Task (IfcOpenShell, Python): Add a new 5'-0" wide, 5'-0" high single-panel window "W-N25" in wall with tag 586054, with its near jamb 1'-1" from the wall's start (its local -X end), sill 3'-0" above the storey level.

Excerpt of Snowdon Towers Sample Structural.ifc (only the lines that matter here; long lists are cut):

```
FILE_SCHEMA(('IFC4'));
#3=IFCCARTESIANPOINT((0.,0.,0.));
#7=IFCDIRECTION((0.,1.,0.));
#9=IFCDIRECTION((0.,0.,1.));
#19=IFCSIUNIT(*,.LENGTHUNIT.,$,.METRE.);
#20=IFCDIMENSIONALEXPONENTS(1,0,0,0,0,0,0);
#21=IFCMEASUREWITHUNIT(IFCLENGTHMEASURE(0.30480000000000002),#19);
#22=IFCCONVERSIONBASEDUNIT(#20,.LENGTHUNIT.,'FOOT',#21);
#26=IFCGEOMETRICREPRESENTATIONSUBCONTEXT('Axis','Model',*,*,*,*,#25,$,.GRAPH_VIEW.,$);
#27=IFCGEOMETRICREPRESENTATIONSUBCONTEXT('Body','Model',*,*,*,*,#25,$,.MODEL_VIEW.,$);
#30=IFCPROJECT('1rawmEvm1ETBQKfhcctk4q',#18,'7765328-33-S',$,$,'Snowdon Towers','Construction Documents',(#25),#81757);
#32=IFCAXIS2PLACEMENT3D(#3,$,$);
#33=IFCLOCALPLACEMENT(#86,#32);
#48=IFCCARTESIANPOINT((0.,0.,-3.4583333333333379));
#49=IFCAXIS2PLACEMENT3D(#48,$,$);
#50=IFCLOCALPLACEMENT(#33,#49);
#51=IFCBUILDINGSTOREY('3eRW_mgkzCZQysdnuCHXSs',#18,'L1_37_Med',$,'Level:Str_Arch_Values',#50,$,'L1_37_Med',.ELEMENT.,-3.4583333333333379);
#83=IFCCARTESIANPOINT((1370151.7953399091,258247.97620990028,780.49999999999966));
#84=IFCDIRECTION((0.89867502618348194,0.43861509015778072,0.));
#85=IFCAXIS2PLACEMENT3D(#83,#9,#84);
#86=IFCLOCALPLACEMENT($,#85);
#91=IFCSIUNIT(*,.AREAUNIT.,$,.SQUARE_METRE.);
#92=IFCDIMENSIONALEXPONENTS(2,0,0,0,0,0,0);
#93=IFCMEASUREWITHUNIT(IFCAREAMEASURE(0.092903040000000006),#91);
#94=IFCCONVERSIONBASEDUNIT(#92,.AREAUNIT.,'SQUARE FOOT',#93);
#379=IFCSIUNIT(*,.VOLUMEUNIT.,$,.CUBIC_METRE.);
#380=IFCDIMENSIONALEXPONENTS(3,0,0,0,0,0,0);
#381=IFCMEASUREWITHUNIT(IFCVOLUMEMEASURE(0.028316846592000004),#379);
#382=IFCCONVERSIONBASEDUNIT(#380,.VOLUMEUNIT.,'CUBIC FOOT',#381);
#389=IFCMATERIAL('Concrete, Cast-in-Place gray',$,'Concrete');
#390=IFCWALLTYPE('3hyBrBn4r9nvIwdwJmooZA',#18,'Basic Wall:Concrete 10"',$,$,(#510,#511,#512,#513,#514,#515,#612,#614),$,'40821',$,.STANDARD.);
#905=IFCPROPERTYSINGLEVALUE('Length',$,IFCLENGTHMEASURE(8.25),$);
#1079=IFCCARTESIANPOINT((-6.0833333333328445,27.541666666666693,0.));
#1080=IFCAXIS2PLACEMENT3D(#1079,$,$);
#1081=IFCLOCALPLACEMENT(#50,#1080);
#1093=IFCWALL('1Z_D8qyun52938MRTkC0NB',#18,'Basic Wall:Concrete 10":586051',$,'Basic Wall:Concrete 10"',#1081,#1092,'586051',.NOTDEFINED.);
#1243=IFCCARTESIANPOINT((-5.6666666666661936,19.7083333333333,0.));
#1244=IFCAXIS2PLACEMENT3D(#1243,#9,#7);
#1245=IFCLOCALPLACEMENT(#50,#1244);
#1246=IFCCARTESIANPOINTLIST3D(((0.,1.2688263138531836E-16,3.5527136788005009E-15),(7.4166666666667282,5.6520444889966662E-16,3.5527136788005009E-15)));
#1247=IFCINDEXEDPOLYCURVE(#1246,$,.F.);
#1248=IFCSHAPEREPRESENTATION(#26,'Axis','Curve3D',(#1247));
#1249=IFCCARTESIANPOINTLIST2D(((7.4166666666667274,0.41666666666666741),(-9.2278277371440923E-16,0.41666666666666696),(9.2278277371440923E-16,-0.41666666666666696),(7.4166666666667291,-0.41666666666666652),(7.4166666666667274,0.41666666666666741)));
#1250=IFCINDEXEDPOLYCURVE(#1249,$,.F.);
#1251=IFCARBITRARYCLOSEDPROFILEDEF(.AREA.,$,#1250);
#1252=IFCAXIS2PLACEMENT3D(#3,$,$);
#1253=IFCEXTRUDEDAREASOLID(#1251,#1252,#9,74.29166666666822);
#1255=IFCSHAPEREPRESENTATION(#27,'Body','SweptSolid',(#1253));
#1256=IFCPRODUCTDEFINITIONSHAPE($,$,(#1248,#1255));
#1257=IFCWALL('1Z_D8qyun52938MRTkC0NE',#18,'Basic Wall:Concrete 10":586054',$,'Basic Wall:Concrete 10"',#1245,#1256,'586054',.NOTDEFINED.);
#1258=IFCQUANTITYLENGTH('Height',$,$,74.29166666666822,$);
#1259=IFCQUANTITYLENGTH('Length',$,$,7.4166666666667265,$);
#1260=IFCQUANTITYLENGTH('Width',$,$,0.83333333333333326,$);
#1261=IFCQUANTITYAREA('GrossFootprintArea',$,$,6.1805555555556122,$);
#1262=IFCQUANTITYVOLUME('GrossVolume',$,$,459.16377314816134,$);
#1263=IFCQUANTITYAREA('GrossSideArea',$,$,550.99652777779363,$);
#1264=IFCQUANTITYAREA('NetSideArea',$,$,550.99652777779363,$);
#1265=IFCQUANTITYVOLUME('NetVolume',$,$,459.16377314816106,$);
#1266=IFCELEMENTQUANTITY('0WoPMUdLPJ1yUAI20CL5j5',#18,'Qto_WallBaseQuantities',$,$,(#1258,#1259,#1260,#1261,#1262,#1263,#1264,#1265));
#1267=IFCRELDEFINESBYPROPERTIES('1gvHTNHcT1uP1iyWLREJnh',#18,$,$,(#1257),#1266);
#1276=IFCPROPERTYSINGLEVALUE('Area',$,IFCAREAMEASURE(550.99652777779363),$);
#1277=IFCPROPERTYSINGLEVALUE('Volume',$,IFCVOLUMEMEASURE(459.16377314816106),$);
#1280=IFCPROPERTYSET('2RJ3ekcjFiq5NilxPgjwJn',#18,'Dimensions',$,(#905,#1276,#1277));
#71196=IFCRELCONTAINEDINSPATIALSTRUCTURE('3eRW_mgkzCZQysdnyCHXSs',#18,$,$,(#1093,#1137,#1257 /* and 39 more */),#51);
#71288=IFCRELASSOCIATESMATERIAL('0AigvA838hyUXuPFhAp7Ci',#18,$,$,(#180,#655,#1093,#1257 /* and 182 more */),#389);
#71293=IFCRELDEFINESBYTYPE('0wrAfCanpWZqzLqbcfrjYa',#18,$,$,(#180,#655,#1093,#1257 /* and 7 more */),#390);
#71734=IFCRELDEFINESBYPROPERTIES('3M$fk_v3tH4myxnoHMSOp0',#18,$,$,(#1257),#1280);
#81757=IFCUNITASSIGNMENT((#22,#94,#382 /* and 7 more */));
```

```python
import numpy as np
import ifcopenshell
import ifcopenshell.api.feature
import ifcopenshell.api.geometry
import ifcopenshell.api.pset
import ifcopenshell.api.root
import ifcopenshell.api.spatial
import ifcopenshell.geom
import ifcopenshell.util.element
import ifcopenshell.util.placement
import ifcopenshell.util.representation
import ifcopenshell.util.shape
import ifcopenshell.util.unit

model = ifcopenshell.open("Snowdon Towers Sample Structural.ifc")
unit_scale = ifcopenshell.util.unit.calculate_unit_scale(model)
area_scale = ifcopenshell.util.unit.calculate_unit_scale(model, "AREAUNIT")
volume_scale = ifcopenshell.util.unit.calculate_unit_scale(model, "VOLUMEUNIT")
settings = ifcopenshell.geom.settings()


def volume(element):
    """Net volume in cubic metres, openings subtracted."""
    shape = ifcopenshell.geom.create_shape(settings, element)
    return ifcopenshell.util.shape.get_volume(shape.geometry)


wall = model.by_id(1257)
storey = ifcopenshell.util.element.get_container(wall, ifc_class="IfcBuildingStorey")
context = ifcopenshell.util.representation.get_context(model, "Model", "Body", "MODEL_VIEW")
before = volume(wall)

width, height, from_end, sill = 1.524, 1.524, 0.3302, 0.9144  # metres

# The wall runs along its own X axis, and the end named is its -X end.
wall_shape = ifcopenshell.geom.create_shape(settings, wall)
x, y, z = ifcopenshell.util.shape.get_vertices(wall_shape.geometry).T
start = x.min() + from_end
face, thickness = float(y.min()), float(y.max() - y.min())
wall_matrix = ifcopenshell.util.placement.get_local_placement(wall.ObjectPlacement)
level = ifcopenshell.util.placement.get_local_placement(storey.ObjectPlacement)[2, 3]


def in_wall(x, y):
    """Placement at x, y metres in the wall's axes, at sill height."""
    matrix = wall_matrix.copy()
    matrix[:, 3] = wall_matrix @ np.array([x / unit_scale, y / unit_scale, 0.0, 1.0])
    matrix[2, 3] = level + sill / unit_scale
    return matrix


# Opening: a box that overshoots both wall faces by 50 mm.
opening = ifcopenshell.api.root.create_entity(model, ifc_class="IfcOpeningElement", predefined_type="OPENING")
box = ifcopenshell.api.geometry.add_wall_representation(
    model, context=context, length=width, height=height, thickness=thickness + 0.1
)
ifcopenshell.api.geometry.assign_representation(model, product=opening, representation=box)
ifcopenshell.api.geometry.edit_object_placement(model, product=opening, matrix=in_wall(start, face - 0.05), is_si=False)
ifcopenshell.api.feature.add_feature(model, feature=opening, element=wall)

window = ifcopenshell.api.root.create_entity(model, ifc_class="IfcWindow", name="W-N25", predefined_type="WINDOW")
window.OverallWidth, window.OverallHeight = width / unit_scale, height / unit_scale
window.PartitioningType = "SINGLE_PANEL"
body = ifcopenshell.api.geometry.add_window_representation(
    model,
    context=context,
    overall_width=window.OverallWidth,
    overall_height=window.OverallHeight,
    partition_type="SINGLE_PANEL",
)
ifcopenshell.api.geometry.assign_representation(model, product=window, representation=body)
ifcopenshell.api.spatial.assign_container(model, products=[window], relating_structure=storey)
ifcopenshell.api.feature.add_filling(model, opening=opening, element=window)

# Centre the window in the wall's thickness.
ifcopenshell.api.geometry.edit_object_placement(model, product=window, matrix=in_wall(start, face), is_si=False)
window_shape = ifcopenshell.geom.create_shape(settings, window)
depth = ifcopenshell.util.shape.get_vertices(window_shape.geometry)[:, 1]
offset = face + thickness / 2 - (depth.min() + depth.max()) / 2
ifcopenshell.api.geometry.edit_object_placement(model, product=window, matrix=in_wall(start, offset), is_si=False)

after = volume(wall)

# Update the wall's stored quantities.
qto = model.by_id(ifcopenshell.util.element.get_pset(wall, "Qto_WallBaseQuantities", should_inherit=False)["id"])
ifcopenshell.api.pset.edit_qto(model, qto=qto, properties={
    "NetSideArea": after / thickness / area_scale,
    "NetVolume": after / volume_scale,
})
pset = model.by_id(ifcopenshell.util.element.get_pset(wall, "Dimensions", should_inherit=False)["id"])
ifcopenshell.api.pset.edit_pset(model, pset=pset, properties={
    "Area": model.create_entity("IfcAreaMeasure", after / thickness / area_scale),
    "Volume": model.create_entity("IfcVolumeMeasure", after / volume_scale),
})

print(f"wall volume {before:.3f} -> {after:.3f} m3")

model.write("Snowdon Towers Sample Structural-out.ifc")
```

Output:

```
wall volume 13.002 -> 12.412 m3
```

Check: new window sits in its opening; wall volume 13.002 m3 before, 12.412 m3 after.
